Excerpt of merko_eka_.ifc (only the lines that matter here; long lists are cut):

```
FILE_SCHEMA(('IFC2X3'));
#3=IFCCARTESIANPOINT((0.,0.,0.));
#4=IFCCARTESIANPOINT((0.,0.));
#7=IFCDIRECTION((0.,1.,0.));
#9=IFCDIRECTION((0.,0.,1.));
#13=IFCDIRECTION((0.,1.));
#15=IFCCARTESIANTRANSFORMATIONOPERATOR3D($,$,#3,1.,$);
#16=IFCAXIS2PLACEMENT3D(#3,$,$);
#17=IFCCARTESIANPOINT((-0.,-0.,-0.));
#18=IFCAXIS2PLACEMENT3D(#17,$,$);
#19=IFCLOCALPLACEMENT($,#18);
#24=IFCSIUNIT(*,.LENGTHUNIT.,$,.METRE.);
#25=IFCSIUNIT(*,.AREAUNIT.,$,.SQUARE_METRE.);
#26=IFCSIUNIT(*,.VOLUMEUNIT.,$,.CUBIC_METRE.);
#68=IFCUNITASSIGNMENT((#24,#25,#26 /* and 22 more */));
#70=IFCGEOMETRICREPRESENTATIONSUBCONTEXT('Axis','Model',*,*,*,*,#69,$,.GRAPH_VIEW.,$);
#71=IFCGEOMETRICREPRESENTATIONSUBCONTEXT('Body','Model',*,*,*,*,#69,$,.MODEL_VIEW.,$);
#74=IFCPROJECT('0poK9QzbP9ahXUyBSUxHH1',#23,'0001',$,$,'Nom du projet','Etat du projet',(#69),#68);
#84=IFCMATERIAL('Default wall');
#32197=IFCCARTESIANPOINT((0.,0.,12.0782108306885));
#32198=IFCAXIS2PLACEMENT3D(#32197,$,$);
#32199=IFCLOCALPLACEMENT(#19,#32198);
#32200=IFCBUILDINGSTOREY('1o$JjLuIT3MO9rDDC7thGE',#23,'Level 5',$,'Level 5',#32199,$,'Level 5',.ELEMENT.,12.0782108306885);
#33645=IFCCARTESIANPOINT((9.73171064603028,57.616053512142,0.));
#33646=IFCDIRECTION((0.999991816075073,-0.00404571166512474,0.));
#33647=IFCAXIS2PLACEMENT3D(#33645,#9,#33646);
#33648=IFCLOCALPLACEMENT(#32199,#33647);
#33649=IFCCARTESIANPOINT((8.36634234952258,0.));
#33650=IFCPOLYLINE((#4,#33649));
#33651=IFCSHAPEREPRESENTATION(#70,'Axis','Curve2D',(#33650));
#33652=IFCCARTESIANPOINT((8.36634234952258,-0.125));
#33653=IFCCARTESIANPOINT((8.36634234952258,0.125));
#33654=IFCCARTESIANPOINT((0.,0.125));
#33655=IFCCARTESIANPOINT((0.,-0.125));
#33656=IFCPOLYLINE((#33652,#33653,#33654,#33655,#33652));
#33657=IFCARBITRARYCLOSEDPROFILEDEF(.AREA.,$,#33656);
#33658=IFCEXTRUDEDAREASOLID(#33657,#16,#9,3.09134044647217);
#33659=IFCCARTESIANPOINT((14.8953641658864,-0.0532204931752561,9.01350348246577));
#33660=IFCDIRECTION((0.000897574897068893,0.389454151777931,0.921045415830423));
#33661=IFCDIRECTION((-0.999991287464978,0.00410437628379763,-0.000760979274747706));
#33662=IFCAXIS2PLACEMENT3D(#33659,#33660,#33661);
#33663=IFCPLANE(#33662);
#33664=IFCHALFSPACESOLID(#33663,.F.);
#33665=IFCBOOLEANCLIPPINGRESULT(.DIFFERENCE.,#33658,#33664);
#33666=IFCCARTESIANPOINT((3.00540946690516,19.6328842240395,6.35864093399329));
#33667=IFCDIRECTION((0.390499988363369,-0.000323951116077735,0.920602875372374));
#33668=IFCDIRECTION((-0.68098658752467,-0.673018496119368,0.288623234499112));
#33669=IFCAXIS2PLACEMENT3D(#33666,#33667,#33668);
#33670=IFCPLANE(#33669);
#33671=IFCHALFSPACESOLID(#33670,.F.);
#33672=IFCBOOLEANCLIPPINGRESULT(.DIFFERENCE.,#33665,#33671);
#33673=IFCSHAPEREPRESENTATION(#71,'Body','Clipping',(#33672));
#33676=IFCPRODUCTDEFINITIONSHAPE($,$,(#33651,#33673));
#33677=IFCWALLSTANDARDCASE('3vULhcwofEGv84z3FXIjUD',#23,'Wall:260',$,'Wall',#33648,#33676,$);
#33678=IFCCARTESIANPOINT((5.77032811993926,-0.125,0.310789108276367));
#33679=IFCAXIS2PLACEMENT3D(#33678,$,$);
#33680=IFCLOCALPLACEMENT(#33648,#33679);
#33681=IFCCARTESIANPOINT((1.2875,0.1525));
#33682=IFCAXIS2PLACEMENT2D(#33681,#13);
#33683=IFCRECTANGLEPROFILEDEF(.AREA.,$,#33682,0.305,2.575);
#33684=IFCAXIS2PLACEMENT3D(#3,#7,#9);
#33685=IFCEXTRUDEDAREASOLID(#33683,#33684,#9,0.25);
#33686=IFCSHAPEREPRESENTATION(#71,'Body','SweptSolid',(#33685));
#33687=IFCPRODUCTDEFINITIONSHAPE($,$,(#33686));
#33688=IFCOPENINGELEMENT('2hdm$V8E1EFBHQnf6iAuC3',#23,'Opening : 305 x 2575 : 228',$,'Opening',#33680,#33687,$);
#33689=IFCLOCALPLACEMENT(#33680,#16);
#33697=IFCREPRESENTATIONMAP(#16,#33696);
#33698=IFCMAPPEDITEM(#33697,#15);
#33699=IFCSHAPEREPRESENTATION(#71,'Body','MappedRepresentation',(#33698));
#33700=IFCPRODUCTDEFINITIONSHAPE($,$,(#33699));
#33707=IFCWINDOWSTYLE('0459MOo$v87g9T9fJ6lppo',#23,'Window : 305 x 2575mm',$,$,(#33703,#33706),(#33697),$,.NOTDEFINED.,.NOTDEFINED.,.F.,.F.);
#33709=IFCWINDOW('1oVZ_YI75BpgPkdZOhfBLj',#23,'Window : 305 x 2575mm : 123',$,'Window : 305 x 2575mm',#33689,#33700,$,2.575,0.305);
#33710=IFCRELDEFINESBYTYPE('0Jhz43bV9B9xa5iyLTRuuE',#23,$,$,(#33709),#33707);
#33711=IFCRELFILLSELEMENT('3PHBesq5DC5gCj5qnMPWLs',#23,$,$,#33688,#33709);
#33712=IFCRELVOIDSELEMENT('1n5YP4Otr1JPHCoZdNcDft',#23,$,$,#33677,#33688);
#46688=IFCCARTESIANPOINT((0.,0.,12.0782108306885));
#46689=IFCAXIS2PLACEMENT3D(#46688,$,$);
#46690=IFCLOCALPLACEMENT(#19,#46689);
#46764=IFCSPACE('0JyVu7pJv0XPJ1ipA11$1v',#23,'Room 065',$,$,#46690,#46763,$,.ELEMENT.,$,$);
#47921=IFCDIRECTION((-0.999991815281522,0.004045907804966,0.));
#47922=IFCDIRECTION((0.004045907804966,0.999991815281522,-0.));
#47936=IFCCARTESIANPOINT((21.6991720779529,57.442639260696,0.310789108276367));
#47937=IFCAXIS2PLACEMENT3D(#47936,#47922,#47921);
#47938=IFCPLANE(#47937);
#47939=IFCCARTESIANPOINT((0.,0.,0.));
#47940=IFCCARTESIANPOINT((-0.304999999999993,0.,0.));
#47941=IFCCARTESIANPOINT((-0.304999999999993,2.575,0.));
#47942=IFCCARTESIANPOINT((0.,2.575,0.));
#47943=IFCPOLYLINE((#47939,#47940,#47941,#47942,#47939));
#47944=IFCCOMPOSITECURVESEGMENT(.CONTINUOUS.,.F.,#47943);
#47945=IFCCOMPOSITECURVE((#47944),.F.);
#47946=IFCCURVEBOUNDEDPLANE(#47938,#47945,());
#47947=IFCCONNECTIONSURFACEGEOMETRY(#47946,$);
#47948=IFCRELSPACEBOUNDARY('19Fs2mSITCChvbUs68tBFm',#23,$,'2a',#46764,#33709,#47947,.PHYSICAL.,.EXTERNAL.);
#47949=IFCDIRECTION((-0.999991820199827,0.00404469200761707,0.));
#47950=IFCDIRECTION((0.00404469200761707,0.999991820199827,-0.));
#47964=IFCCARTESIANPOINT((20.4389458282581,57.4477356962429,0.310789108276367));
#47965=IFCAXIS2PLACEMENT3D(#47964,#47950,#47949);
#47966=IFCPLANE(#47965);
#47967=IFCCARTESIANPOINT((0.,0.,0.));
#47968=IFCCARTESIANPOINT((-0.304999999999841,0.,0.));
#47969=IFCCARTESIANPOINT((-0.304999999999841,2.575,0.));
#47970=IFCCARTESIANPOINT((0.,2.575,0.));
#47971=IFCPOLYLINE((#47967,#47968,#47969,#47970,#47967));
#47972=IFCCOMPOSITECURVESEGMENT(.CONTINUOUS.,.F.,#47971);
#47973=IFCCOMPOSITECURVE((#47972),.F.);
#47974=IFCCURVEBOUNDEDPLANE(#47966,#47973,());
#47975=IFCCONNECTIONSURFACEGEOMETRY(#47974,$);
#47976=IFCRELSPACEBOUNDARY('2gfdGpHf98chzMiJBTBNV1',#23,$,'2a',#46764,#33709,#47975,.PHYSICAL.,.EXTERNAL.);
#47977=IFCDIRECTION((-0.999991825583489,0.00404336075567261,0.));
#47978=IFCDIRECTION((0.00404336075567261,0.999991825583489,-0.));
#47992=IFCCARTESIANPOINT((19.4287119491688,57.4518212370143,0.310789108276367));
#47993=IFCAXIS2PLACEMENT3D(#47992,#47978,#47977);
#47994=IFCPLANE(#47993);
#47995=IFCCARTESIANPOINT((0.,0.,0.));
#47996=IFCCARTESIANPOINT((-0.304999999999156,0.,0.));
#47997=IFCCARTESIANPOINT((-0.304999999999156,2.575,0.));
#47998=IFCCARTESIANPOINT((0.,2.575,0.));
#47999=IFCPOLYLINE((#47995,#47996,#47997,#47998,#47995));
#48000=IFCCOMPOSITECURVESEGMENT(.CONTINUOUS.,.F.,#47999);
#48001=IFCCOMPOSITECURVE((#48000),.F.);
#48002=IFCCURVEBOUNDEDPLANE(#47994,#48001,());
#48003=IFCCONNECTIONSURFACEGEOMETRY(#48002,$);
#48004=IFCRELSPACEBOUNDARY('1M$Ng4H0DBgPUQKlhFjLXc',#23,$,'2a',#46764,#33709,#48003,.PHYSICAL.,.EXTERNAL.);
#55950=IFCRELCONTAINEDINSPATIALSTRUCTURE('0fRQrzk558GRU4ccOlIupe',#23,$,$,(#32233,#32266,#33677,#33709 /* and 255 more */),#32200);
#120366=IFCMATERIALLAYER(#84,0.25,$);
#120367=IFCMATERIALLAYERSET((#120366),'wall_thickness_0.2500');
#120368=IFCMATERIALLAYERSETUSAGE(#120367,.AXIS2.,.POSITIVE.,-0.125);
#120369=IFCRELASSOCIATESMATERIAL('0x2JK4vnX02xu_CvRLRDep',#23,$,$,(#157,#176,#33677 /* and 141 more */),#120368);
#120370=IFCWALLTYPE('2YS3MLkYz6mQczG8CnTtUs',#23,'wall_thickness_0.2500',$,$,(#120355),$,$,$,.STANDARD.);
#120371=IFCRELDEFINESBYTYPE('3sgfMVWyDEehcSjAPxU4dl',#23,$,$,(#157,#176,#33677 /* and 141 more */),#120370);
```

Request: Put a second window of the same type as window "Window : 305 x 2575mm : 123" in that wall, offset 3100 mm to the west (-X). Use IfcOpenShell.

```python
import numpy as np
import ifcopenshell
import ifcopenshell.api.feature
import ifcopenshell.api.geometry
import ifcopenshell.api.root
import ifcopenshell.geom
import ifcopenshell.util.element
import ifcopenshell.util.placement
import ifcopenshell.util.shape

model = ifcopenshell.open("merko_eka_.ifc")
settings = ifcopenshell.geom.settings()


def volume(element):
    """Net volume in cubic metres, openings subtracted."""
    shape = ifcopenshell.geom.create_shape(settings, element)
    return ifcopenshell.util.shape.get_volume(shape.geometry)


window = model.by_guid("1oVZ_YI75BpgPkdZOhfBLj")
opening = window.FillsVoids[0].RelatingOpeningElement
wall = opening.VoidsElements[0].RelatingBuildingElement
before = volume(wall)
shift = ifcopenshell.util.placement.get_local_placement(wall.ObjectPlacement)[:3, 0] * -3.1

# copy_class copies the void relationship, type, container and properties, but no geometry.
new_opening = ifcopenshell.api.root.copy_class(model, product=opening)
new_opening.Representation = ifcopenshell.util.element.copy_deep(
    model, opening.Representation, exclude=["IfcGeometricRepresentationContext", "IfcRepresentationMap"]
)
new_opening.Name = "Opening : 305 x 2575"
new_window = ifcopenshell.api.root.copy_class(model, product=window)
new_window.Representation = ifcopenshell.util.element.copy_deep(
    model, window.Representation, exclude=["IfcGeometricRepresentationContext", "IfcRepresentationMap"]
)
new_window.Name = "Window : 305 x 2575mm"
fills = ifcopenshell.api.feature.add_filling(model, opening=new_opening, element=new_window)
fills.OwnerHistory = new_window.OwnerHistory  # required in IFC2X3

for old, new in ((opening, new_opening), (window, new_window)):
    matrix = ifcopenshell.util.placement.get_local_placement(old.ObjectPlacement)
    matrix[:3, 3] += shift
    ifcopenshell.api.geometry.edit_object_placement(model, product=new, matrix=matrix, is_si=False)

# The copied space boundaries still share their surfaces with the original.
for rel in new_window.ProvidesBoundaries:
    if rel.ConnectionGeometry:
        rel.ConnectionGeometry = ifcopenshell.util.element.copy_deep(model, rel.ConnectionGeometry)

# Space boundary surfaces are stored in each space's coordinates; move them too.
for rel in new_window.ProvidesBoundaries:
    if not rel.ConnectionGeometry:
        continue
    surface = rel.ConnectionGeometry.SurfaceOnRelatingElement.BasisSurface
    space_matrix = ifcopenshell.util.placement.get_local_placement(rel.RelatingSpace.ObjectPlacement)
    point = np.array(surface.Position.Location.Coordinates) + space_matrix[:3, :3].T @ shift
    surface.Position = model.createIfcAxis2Placement3D(
        model.createIfcCartesianPoint(point.tolist()), surface.Position.Axis, surface.Position.RefDirection
    )

after = volume(wall)

print(f"wall volume {before:.3f} -> {after:.3f} m3")

model.write("merko_eka__rev.ifc")
```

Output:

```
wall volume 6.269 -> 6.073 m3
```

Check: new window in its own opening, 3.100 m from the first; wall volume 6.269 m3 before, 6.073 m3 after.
